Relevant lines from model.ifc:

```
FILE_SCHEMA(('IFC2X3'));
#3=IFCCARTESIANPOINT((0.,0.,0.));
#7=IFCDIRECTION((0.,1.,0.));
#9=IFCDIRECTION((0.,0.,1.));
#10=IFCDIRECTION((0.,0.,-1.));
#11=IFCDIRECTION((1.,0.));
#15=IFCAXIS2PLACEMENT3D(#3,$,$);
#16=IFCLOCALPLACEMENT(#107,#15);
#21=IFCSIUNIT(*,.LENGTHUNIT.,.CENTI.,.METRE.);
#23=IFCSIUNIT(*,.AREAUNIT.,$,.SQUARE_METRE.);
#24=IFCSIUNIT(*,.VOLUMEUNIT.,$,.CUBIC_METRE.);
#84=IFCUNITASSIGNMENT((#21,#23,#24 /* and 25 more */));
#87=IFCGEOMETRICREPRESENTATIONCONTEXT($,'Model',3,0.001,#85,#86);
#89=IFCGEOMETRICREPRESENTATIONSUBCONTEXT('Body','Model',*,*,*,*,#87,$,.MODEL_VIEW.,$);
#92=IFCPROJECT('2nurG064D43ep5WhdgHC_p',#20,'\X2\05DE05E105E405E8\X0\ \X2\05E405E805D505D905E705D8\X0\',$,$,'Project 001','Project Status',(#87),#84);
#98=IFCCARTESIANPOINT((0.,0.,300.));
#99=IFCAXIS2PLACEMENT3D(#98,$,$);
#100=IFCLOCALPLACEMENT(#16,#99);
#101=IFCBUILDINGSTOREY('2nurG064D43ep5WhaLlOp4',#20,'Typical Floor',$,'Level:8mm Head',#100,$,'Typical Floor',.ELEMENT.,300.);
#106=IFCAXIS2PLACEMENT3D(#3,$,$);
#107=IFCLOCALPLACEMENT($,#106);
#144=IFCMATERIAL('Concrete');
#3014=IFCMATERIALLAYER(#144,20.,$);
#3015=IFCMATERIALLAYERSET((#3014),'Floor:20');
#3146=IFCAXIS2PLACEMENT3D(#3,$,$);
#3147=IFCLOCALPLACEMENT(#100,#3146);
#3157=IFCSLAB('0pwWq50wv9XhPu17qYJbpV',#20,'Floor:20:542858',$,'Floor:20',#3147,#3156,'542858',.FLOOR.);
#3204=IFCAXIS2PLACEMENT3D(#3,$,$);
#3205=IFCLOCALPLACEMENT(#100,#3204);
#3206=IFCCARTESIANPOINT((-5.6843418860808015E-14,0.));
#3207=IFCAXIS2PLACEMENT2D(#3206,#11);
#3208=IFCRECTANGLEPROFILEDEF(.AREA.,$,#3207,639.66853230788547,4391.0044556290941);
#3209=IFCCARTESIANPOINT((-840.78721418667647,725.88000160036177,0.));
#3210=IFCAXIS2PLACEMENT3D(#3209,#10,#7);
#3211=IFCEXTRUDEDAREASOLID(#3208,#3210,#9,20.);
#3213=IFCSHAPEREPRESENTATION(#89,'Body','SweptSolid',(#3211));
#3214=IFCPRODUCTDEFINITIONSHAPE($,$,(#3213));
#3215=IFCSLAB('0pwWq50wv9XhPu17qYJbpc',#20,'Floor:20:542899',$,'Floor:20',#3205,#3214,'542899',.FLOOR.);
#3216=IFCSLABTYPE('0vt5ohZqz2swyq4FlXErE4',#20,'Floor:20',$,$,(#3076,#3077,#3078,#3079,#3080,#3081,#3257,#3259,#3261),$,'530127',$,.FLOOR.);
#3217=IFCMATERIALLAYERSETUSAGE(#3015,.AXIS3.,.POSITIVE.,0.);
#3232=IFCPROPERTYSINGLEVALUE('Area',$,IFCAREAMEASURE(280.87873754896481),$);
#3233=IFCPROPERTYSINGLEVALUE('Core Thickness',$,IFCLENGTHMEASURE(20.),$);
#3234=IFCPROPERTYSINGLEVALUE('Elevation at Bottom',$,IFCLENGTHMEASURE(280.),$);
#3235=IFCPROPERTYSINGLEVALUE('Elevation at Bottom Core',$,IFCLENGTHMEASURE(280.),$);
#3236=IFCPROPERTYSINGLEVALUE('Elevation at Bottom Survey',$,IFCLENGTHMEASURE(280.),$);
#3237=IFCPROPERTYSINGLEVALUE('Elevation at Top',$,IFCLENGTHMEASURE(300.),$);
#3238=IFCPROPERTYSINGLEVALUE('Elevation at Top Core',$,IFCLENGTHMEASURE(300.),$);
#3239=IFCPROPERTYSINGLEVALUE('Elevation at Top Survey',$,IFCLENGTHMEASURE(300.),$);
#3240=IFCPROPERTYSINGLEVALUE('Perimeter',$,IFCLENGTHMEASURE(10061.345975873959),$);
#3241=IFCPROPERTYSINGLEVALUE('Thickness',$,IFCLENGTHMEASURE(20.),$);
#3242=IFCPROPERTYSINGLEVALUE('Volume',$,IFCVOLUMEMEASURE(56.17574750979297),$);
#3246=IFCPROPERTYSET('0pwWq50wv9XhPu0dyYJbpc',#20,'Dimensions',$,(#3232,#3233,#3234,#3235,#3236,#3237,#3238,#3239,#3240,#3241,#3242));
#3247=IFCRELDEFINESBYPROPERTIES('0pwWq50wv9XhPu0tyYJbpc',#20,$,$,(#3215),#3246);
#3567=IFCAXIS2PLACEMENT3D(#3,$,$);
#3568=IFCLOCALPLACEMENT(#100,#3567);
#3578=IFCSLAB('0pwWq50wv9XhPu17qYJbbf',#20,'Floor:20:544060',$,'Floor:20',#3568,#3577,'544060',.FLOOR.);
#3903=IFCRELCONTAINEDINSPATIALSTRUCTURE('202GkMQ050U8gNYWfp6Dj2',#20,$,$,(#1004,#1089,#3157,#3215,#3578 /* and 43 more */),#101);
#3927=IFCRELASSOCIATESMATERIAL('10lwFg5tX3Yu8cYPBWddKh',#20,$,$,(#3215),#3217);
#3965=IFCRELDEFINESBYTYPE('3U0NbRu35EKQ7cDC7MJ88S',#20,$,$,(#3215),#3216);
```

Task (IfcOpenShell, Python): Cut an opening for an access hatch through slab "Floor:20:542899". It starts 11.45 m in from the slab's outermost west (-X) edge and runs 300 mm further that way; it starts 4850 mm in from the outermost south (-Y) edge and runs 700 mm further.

```python
import numpy as np
import ifcopenshell
import ifcopenshell.api.feature
import ifcopenshell.api.geometry
import ifcopenshell.api.pset
import ifcopenshell.api.root
import ifcopenshell.geom
import ifcopenshell.util.element
import ifcopenshell.util.placement
import ifcopenshell.util.representation
import ifcopenshell.util.shape
import ifcopenshell.util.unit

model = ifcopenshell.open("model.ifc")
unit_scale = ifcopenshell.util.unit.calculate_unit_scale(model)
area_scale = ifcopenshell.util.unit.calculate_unit_scale(model, "AREAUNIT")
volume_scale = ifcopenshell.util.unit.calculate_unit_scale(model, "VOLUMEUNIT")
settings = ifcopenshell.geom.settings()


def volume(element):
    """Net volume in cubic metres, openings subtracted."""
    shape = ifcopenshell.geom.create_shape(settings, element)
    return ifcopenshell.util.shape.get_volume(shape.geometry)


slab = model.by_guid("0pwWq50wv9XhPu17qYJbpc")
before = volume(slab)

# Extent in the slab's own axes, in metres. The edges named are its -X and -Y sides.
slab_shape = ifcopenshell.geom.create_shape(settings, slab)
vertices = ifcopenshell.util.shape.get_vertices(slab_shape.geometry)
x_min, y_min, bottom = vertices.min(axis=0)
top = vertices[:, 2].max()

opening = ifcopenshell.api.root.create_entity(model, ifc_class="IfcOpeningElement", name="Access hatch opening")
context = ifcopenshell.util.representation.get_context(model, "Model", "Body", "MODEL_VIEW")
width, depth = 0.3, 0.7
outline = [(0.0, 0.0), (width, 0.0), (width, depth), (0.0, depth), (0.0, 0.0)]
# Overshoot both faces by 50 mm so the cut is clean.
shape = ifcopenshell.api.geometry.add_slab_representation(
    model, context=context, depth=top - bottom + 0.1, polyline=outline
)
ifcopenshell.api.geometry.assign_representation(model, product=opening, representation=shape)

matrix = ifcopenshell.util.placement.get_local_placement(slab.ObjectPlacement)
matrix[:, 3] = matrix @ np.append(np.array([x_min + 11.45, y_min + 4.85, bottom - 0.05]) / unit_scale, 1.0)
ifcopenshell.api.geometry.edit_object_placement(model, product=opening, matrix=matrix, is_si=False)
ifcopenshell.api.feature.add_feature(model, feature=opening, element=slab)

after = volume(slab)

# Update the slab's stored quantities.
pset = model.by_id(ifcopenshell.util.element.get_pset(slab, "Dimensions", should_inherit=False)["id"])
ifcopenshell.api.pset.edit_pset(model, pset=pset, properties={
    "Area": model.create_entity("IfcAreaMeasure", after / (top - bottom) / area_scale),
    "Volume": model.create_entity("IfcVolumeMeasure", after / volume_scale),
})

print(f"slab volume {before:.3f} -> {after:.3f} m3")

model.write("model-out.ifc")
```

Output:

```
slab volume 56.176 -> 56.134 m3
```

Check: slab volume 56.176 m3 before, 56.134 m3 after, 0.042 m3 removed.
